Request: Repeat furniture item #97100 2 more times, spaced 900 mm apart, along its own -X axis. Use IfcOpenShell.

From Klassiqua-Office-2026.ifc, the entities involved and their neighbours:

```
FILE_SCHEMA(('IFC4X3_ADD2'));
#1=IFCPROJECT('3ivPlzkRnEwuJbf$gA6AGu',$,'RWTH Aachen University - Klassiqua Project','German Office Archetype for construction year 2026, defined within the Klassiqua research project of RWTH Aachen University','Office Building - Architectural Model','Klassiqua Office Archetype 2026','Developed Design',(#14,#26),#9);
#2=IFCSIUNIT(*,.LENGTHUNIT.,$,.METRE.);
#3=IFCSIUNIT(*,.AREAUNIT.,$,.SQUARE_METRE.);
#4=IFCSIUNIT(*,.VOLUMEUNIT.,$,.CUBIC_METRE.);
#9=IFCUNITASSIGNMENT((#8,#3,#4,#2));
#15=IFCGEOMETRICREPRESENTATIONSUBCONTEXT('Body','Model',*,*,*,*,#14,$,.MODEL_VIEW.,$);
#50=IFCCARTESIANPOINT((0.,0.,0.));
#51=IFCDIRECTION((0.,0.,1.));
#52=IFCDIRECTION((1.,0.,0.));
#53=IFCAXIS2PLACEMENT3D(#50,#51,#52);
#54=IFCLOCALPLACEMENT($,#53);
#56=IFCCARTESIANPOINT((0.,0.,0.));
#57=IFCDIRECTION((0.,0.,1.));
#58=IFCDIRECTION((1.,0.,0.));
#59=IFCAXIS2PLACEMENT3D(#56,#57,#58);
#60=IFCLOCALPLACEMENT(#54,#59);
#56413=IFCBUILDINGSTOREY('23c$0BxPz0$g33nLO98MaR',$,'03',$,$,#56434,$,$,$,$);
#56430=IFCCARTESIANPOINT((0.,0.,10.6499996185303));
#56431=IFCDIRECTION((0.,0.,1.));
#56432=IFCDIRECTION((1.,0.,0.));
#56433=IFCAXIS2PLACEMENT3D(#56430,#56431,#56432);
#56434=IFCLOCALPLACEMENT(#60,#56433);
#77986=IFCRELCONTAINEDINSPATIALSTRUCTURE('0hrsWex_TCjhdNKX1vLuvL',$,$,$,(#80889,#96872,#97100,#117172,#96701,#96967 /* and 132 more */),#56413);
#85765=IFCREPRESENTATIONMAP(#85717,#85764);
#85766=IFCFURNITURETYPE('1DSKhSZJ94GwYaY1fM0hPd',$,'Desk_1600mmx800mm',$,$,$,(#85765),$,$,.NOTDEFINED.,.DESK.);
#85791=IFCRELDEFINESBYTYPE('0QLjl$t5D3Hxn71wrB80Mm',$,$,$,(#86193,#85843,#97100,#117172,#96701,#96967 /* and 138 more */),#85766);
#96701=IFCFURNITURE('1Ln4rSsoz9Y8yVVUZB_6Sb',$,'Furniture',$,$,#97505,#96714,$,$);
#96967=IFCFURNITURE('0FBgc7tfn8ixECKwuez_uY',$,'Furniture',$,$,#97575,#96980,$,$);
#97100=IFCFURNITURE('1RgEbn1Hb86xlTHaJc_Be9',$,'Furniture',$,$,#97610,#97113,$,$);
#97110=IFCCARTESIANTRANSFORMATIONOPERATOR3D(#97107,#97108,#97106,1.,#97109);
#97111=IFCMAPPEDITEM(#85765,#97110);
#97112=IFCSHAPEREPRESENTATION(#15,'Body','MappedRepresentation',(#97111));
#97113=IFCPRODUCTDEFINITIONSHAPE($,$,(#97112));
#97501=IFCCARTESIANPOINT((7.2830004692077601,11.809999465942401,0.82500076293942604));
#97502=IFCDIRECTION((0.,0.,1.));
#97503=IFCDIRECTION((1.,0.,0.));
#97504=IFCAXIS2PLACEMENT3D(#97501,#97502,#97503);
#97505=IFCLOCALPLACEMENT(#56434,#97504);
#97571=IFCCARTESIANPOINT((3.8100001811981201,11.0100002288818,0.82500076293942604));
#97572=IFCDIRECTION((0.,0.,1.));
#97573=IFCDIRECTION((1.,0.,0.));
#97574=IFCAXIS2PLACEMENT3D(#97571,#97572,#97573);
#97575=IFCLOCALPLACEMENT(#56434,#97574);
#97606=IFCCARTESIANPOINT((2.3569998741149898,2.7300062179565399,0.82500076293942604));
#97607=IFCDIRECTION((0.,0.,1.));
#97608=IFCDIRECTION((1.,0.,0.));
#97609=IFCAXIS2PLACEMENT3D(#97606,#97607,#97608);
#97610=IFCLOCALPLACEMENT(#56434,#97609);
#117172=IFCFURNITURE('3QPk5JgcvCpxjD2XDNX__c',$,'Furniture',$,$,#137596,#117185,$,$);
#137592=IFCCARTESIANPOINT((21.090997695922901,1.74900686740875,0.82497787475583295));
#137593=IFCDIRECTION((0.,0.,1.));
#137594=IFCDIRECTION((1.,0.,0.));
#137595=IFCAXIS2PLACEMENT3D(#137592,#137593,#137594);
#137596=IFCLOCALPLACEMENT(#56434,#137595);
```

```python
import ifcopenshell
import ifcopenshell.api.geometry
import ifcopenshell.api.root
import ifcopenshell.util.element
import ifcopenshell.util.placement
import ifcopenshell.util.unit

model = ifcopenshell.open("Klassiqua-Office-2026.ifc")
unit_scale = ifcopenshell.util.unit.calculate_unit_scale(model)

source = model.by_guid("1RgEbn1Hb86xlTHaJc_Be9")
base = ifcopenshell.util.placement.get_local_placement(source.ObjectPlacement)
step = -base[:3, 0] * 0.9 / unit_scale

for i in range(1, 3):
    copy = ifcopenshell.api.root.copy_class(model, product=source)
    copy.Representation = ifcopenshell.util.element.copy_deep(
        model, source.Representation, exclude=["IfcGeometricRepresentationContext", "IfcRepresentationMap"]
    )
    matrix = base.copy()
    matrix[:3, 3] += i * step
    print("added at", matrix[:3, 3].round(3) + 0.0)
    ifcopenshell.api.geometry.edit_object_placement(model, product=copy, matrix=matrix, is_si=False)

model.write("Klassiqua-Office-2026_updated.ifc")
```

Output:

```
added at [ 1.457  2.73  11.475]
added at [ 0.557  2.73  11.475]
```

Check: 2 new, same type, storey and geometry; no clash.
